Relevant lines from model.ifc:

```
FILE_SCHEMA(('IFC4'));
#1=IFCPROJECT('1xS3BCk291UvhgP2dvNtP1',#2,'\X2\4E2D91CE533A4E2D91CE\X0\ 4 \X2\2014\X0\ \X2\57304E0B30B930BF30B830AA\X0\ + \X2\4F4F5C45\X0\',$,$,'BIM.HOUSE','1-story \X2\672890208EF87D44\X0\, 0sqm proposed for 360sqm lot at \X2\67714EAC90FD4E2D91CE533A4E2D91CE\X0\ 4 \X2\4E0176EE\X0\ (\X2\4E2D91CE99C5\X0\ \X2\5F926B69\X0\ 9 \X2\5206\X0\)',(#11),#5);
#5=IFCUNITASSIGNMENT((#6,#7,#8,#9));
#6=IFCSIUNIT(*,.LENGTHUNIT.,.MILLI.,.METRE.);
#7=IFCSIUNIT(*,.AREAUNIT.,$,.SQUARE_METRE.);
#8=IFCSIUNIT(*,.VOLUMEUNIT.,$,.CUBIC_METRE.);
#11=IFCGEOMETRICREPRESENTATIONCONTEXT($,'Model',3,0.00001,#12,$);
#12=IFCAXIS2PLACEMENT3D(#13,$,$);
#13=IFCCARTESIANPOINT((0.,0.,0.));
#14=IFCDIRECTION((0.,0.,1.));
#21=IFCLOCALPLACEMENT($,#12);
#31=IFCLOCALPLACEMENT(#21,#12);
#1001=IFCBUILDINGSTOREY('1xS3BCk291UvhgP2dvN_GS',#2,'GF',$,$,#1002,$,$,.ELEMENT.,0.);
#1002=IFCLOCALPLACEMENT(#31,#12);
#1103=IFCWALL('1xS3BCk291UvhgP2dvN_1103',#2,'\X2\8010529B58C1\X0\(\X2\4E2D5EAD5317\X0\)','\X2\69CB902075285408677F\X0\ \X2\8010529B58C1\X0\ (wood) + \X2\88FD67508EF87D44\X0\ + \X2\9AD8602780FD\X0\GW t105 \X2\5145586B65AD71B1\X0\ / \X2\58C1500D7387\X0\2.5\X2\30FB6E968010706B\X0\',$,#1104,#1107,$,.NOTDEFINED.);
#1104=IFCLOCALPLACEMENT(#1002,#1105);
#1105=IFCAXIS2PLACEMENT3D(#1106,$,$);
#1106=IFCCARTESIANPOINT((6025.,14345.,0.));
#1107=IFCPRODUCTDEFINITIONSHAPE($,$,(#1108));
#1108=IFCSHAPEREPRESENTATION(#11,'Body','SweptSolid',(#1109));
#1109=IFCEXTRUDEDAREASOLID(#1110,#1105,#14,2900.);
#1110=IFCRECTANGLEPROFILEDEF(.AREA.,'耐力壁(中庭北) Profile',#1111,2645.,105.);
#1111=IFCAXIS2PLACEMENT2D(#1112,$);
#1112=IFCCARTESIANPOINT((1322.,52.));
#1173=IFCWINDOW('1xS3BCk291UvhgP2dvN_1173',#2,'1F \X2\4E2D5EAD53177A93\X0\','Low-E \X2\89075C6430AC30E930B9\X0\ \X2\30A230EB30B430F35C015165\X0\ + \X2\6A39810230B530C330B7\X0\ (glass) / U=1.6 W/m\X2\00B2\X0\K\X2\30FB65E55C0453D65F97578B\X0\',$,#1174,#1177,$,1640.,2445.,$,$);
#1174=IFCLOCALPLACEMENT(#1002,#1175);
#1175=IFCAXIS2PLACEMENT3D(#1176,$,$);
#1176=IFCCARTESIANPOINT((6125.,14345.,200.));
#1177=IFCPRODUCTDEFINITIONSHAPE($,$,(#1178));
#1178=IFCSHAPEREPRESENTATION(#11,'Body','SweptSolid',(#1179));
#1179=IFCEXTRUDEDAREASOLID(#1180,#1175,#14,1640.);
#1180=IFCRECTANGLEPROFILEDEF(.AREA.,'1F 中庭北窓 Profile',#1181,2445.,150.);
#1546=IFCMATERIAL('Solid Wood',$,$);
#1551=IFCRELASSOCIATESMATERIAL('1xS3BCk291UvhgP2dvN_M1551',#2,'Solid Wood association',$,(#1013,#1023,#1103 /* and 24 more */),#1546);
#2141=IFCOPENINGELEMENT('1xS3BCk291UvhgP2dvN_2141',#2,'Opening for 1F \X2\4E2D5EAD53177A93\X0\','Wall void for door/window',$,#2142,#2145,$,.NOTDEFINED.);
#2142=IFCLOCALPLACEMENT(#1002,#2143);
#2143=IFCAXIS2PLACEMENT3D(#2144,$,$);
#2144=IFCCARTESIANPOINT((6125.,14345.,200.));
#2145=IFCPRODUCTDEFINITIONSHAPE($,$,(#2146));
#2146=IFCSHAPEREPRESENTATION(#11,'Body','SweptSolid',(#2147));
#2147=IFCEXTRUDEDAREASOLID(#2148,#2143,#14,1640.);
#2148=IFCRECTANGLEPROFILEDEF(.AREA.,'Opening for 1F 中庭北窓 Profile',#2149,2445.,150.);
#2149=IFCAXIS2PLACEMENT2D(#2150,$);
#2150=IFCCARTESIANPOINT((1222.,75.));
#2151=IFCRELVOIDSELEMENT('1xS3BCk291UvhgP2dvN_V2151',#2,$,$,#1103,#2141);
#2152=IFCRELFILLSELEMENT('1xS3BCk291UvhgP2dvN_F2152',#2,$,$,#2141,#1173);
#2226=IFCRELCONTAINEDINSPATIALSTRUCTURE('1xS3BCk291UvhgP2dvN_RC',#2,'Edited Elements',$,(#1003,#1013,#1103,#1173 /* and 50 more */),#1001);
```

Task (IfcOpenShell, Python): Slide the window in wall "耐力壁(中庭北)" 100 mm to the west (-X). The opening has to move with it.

```python
import ifcopenshell
import ifcopenshell.api.geometry
import ifcopenshell.util.placement

model = ifcopenshell.open("model.ifc")

window = model.by_guid("1xS3BCk291UvhgP2dvN_1173")
opening = window.FillsVoids[0].RelatingOpeningElement
wall = opening.VoidsElements[0].RelatingBuildingElement

wall_matrix = ifcopenshell.util.placement.get_local_placement(wall.ObjectPlacement)
shift = wall_matrix[:3, 0] * -100.0
before = ifcopenshell.util.placement.get_local_placement(window.ObjectPlacement)[:3, 3].copy()

# The window is not placed relative to its opening, so move both.
for product in (opening, window):
    matrix = ifcopenshell.util.placement.get_local_placement(product.ObjectPlacement)
    matrix[:3, 3] += shift
    ifcopenshell.api.geometry.edit_object_placement(model, product=product, matrix=matrix, is_si=False)

after = ifcopenshell.util.placement.get_local_placement(window.ObjectPlacement)[:3, 3]
print("window moved by", (after - before).round(3) + 0.0)

model.write("model_rev.ifc")
```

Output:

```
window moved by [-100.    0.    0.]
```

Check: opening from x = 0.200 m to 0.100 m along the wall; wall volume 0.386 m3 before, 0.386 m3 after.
